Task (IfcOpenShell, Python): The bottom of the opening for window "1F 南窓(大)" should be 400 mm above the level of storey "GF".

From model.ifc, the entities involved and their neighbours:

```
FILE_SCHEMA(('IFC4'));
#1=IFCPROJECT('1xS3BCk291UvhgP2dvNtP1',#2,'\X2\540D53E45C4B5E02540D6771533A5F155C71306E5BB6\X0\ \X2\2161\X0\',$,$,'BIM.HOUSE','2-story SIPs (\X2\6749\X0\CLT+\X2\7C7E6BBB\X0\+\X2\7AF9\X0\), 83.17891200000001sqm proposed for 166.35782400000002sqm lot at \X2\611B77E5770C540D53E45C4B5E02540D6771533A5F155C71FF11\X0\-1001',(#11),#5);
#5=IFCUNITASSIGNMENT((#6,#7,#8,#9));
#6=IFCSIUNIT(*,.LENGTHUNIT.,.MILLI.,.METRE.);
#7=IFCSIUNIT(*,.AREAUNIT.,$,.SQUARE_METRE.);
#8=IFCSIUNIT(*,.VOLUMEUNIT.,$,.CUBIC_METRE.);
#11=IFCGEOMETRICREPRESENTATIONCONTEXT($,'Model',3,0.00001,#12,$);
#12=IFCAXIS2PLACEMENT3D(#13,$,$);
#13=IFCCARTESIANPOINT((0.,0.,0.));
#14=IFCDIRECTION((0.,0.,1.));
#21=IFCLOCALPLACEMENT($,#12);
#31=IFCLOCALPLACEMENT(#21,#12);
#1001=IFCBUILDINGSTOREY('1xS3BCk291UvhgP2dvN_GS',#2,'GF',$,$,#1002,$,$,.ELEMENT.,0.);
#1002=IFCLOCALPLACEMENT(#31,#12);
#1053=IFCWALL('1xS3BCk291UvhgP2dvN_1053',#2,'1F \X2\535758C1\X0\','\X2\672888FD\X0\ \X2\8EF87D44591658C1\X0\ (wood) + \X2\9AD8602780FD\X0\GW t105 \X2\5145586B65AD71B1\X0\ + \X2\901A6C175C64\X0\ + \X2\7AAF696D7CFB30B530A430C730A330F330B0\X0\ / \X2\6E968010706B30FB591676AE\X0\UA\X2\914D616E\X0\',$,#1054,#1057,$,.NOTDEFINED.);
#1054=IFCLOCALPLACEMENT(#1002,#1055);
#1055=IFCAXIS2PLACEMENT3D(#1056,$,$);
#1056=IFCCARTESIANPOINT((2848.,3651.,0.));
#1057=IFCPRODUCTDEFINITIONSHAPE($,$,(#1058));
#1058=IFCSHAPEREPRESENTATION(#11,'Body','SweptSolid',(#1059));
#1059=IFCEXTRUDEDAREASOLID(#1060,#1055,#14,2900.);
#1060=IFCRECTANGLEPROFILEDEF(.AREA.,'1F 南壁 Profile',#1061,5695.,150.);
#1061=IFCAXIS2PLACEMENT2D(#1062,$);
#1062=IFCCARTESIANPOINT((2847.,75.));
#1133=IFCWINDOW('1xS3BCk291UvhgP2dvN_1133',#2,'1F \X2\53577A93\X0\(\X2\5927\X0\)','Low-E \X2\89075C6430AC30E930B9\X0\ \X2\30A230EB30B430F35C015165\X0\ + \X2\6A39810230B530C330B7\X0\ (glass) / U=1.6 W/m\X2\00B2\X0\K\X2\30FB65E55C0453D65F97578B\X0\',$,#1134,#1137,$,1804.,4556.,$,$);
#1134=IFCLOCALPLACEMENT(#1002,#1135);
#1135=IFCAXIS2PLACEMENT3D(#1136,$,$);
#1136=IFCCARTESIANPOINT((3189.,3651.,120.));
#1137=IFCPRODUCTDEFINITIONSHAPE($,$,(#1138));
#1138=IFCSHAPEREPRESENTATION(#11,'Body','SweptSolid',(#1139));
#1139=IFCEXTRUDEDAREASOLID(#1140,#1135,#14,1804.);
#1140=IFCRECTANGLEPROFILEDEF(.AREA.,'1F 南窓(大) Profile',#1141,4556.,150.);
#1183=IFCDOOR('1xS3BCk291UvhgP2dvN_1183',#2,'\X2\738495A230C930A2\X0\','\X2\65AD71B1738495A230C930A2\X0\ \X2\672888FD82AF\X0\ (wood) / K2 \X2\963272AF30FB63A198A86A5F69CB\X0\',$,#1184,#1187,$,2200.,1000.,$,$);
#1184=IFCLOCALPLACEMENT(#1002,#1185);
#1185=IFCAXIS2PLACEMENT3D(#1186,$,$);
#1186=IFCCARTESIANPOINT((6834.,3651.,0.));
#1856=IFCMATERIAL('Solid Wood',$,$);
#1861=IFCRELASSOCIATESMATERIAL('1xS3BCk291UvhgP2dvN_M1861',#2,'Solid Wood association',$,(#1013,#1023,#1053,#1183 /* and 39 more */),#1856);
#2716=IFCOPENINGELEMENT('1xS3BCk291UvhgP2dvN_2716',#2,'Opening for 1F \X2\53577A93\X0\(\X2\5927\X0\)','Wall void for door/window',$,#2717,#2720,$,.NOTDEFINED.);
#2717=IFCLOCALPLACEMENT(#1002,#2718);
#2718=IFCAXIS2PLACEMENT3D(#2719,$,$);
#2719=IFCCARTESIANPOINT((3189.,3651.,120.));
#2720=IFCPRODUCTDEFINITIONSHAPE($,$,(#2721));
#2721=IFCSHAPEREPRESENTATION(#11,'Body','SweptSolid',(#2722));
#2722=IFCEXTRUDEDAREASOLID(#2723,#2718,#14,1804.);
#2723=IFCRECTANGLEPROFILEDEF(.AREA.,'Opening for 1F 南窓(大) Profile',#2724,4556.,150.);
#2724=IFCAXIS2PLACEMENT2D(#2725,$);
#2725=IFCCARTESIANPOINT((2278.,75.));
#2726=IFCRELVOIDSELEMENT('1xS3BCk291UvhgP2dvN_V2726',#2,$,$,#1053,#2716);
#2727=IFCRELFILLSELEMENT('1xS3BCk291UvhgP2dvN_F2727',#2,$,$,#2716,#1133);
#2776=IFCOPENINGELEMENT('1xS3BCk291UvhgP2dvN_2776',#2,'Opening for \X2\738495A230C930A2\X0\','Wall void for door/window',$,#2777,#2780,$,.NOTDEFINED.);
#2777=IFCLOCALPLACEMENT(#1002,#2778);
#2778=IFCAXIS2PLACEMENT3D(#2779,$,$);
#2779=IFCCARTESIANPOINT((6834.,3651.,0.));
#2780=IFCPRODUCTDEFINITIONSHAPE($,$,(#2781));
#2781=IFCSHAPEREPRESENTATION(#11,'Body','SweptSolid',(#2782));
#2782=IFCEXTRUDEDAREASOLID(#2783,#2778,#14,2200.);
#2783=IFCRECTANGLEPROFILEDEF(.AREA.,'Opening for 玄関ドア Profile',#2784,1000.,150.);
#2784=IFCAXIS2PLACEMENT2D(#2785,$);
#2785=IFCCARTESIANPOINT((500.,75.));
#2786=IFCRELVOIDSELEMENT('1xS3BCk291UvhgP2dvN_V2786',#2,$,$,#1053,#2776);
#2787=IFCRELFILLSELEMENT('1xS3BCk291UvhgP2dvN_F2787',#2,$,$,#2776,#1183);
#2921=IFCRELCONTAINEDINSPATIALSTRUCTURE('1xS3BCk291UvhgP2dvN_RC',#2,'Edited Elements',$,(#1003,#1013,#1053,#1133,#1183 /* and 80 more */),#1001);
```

```python
import numpy as np
import ifcopenshell
import ifcopenshell.api.geometry
import ifcopenshell.geom
import ifcopenshell.util.element
import ifcopenshell.util.placement
import ifcopenshell.util.shape
import ifcopenshell.util.unit

model = ifcopenshell.open("model.ifc")
unit_scale = ifcopenshell.util.unit.calculate_unit_scale(model)

window = model.by_id(1133)
opening = window.FillsVoids[0].RelatingOpeningElement
storey = ifcopenshell.util.element.get_container(window, ifc_class="IfcBuildingStorey")
level = ifcopenshell.util.placement.get_local_placement(storey.ObjectPlacement)[2, 3]

# The opening's origin need not be at the sill, so measure its lowest point.
shape = ifcopenshell.geom.create_shape(ifcopenshell.geom.settings(), opening)
bottom = ifcopenshell.util.shape.get_shape_bottom_elevation(shape, shape.geometry) / unit_scale
dz = level + 400.0 - bottom

shift = np.array([0.0, 0.0, dz])
# The window is not placed relative to its opening, so move both.
for product in (opening, window):
    matrix = ifcopenshell.util.placement.get_local_placement(product.ObjectPlacement)
    matrix[:3, 3] += shift
    ifcopenshell.api.geometry.edit_object_placement(model, product=product, matrix=matrix, is_si=False)

print(f"moved by {dz * unit_scale:+.3f} m")

model.write("model-out.ifc")
```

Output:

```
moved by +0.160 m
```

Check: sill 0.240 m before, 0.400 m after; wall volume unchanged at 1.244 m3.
